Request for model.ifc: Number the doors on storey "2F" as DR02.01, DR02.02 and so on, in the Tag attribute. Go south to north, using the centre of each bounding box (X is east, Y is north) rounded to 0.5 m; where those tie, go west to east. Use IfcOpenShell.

First a look at what the model holds.

```python
import ifcopenshell
import ifcopenshell.util.element
import ifcopenshell.util.placement

model = ifcopenshell.open("model.ifc")
print(model.schema)
storey = next(s for s in model.by_type("IfcBuildingStorey") if s.Name == "2F")
doors = [e for e in ifcopenshell.util.element.get_decomposition(storey) if e.is_a("IfcDoor")]
for e in sorted(doors, key=lambda e: e.id()):
    origin = ifcopenshell.util.placement.get_local_placement(e.ObjectPlacement)[:3, 3]
    print(e.id(), e.Tag, e.Name, origin.round(2) + 0.0, sep=" | ")
```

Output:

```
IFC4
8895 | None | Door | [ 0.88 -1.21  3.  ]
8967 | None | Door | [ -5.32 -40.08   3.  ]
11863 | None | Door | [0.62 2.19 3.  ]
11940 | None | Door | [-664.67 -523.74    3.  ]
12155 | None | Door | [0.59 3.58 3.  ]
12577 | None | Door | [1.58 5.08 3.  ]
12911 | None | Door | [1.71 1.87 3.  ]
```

```python
import ifcopenshell
import ifcopenshell.geom
import ifcopenshell.util.element
import ifcopenshell.util.shape

model = ifcopenshell.open("model.ifc")
settings = ifcopenshell.geom.settings()
settings.set("use-world-coords", True)


def centre(element):
    shape = ifcopenshell.geom.create_shape(settings, element)
    return ifcopenshell.util.shape.get_bbox_centroid(shape.geometry)


storey = next(s for s in model.by_type("IfcBuildingStorey") if s.Name == "2F")
doors = [e for e in ifcopenshell.util.element.get_decomposition(storey) if e.is_a("IfcDoor")]

# Insertion points can sit at a corner or the storey origin, so sort by the geometry (in metres).
centres = {e: centre(e) for e in doors}
doors.sort(key=lambda e: (round(centres[e][1] / 0.5), centres[e][0]))

for i, e in enumerate(doors, start=1):
    number = f"DR02.{i:02d}"
    e.Tag = number
    print(e.id(), number)

model.write("model_v2.ifc")
```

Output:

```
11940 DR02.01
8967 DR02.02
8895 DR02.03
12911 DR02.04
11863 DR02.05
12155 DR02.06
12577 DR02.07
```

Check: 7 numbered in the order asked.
